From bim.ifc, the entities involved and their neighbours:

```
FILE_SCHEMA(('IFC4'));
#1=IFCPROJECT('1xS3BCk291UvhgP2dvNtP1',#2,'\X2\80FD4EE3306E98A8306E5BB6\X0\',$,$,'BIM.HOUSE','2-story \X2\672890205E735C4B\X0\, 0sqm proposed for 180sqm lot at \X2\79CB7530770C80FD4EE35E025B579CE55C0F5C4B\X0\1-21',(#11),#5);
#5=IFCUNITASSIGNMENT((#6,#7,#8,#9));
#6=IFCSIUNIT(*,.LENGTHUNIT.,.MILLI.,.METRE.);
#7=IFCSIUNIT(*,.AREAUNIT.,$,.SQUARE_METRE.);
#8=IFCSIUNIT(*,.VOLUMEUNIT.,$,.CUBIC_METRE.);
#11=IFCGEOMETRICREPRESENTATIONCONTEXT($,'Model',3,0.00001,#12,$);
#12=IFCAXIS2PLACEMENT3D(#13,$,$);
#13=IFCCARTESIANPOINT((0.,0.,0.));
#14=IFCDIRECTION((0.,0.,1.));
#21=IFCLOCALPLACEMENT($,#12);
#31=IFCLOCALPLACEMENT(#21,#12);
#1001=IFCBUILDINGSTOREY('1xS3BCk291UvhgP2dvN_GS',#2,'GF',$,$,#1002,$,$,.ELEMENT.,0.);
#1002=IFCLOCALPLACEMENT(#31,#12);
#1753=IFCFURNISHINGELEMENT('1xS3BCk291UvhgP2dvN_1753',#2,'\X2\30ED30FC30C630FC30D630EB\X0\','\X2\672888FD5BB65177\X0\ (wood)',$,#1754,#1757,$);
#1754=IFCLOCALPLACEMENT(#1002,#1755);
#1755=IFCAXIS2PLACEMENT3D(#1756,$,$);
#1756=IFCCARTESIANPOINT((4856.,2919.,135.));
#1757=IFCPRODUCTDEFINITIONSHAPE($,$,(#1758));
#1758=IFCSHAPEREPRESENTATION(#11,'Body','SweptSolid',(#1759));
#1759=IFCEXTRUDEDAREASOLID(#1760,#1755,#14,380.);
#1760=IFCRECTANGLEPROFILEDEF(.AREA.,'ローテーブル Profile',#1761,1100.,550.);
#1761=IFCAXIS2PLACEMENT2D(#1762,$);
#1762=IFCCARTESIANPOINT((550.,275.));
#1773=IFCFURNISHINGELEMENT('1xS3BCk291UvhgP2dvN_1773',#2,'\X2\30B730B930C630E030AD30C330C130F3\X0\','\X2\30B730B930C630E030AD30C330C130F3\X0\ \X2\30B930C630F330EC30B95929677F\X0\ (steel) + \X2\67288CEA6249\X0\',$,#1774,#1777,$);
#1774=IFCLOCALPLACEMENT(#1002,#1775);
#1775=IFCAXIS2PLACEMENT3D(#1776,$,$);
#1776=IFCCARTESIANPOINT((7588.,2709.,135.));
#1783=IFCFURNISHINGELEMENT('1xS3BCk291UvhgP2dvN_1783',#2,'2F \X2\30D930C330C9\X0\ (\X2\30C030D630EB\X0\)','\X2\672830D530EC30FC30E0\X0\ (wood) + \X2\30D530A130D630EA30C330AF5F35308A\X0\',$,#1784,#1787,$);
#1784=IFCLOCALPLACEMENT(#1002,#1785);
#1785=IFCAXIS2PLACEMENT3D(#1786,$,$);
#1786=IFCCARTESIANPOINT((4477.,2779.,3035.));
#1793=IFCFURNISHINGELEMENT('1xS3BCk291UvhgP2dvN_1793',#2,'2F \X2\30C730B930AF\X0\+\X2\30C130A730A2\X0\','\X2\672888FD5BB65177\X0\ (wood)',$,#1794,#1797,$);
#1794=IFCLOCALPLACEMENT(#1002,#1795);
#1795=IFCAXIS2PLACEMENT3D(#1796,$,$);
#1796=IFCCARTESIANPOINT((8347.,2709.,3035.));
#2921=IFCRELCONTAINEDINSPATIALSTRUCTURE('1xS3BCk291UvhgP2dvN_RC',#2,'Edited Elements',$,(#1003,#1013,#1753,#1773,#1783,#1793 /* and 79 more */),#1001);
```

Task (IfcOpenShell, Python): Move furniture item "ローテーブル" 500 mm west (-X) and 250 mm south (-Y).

```python
import ifcopenshell
import ifcopenshell.api.geometry
import ifcopenshell.util.placement

model = ifcopenshell.open("bim.ifc")

item = model.by_id(1753)
matrix = ifcopenshell.util.placement.get_local_placement(item.ObjectPlacement)
matrix[0, 3] -= 500.0
matrix[1, 3] -= 250.0
ifcopenshell.api.geometry.edit_object_placement(model, product=item, matrix=matrix, is_si=False)

print(ifcopenshell.util.placement.get_local_placement(item.ObjectPlacement).round(3) + 0.0)

model.write("bim_rev.ifc")
```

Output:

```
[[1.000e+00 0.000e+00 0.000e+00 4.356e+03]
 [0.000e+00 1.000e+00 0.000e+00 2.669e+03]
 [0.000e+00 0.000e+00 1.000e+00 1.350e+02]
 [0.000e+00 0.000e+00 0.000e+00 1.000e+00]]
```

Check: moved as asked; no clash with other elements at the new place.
